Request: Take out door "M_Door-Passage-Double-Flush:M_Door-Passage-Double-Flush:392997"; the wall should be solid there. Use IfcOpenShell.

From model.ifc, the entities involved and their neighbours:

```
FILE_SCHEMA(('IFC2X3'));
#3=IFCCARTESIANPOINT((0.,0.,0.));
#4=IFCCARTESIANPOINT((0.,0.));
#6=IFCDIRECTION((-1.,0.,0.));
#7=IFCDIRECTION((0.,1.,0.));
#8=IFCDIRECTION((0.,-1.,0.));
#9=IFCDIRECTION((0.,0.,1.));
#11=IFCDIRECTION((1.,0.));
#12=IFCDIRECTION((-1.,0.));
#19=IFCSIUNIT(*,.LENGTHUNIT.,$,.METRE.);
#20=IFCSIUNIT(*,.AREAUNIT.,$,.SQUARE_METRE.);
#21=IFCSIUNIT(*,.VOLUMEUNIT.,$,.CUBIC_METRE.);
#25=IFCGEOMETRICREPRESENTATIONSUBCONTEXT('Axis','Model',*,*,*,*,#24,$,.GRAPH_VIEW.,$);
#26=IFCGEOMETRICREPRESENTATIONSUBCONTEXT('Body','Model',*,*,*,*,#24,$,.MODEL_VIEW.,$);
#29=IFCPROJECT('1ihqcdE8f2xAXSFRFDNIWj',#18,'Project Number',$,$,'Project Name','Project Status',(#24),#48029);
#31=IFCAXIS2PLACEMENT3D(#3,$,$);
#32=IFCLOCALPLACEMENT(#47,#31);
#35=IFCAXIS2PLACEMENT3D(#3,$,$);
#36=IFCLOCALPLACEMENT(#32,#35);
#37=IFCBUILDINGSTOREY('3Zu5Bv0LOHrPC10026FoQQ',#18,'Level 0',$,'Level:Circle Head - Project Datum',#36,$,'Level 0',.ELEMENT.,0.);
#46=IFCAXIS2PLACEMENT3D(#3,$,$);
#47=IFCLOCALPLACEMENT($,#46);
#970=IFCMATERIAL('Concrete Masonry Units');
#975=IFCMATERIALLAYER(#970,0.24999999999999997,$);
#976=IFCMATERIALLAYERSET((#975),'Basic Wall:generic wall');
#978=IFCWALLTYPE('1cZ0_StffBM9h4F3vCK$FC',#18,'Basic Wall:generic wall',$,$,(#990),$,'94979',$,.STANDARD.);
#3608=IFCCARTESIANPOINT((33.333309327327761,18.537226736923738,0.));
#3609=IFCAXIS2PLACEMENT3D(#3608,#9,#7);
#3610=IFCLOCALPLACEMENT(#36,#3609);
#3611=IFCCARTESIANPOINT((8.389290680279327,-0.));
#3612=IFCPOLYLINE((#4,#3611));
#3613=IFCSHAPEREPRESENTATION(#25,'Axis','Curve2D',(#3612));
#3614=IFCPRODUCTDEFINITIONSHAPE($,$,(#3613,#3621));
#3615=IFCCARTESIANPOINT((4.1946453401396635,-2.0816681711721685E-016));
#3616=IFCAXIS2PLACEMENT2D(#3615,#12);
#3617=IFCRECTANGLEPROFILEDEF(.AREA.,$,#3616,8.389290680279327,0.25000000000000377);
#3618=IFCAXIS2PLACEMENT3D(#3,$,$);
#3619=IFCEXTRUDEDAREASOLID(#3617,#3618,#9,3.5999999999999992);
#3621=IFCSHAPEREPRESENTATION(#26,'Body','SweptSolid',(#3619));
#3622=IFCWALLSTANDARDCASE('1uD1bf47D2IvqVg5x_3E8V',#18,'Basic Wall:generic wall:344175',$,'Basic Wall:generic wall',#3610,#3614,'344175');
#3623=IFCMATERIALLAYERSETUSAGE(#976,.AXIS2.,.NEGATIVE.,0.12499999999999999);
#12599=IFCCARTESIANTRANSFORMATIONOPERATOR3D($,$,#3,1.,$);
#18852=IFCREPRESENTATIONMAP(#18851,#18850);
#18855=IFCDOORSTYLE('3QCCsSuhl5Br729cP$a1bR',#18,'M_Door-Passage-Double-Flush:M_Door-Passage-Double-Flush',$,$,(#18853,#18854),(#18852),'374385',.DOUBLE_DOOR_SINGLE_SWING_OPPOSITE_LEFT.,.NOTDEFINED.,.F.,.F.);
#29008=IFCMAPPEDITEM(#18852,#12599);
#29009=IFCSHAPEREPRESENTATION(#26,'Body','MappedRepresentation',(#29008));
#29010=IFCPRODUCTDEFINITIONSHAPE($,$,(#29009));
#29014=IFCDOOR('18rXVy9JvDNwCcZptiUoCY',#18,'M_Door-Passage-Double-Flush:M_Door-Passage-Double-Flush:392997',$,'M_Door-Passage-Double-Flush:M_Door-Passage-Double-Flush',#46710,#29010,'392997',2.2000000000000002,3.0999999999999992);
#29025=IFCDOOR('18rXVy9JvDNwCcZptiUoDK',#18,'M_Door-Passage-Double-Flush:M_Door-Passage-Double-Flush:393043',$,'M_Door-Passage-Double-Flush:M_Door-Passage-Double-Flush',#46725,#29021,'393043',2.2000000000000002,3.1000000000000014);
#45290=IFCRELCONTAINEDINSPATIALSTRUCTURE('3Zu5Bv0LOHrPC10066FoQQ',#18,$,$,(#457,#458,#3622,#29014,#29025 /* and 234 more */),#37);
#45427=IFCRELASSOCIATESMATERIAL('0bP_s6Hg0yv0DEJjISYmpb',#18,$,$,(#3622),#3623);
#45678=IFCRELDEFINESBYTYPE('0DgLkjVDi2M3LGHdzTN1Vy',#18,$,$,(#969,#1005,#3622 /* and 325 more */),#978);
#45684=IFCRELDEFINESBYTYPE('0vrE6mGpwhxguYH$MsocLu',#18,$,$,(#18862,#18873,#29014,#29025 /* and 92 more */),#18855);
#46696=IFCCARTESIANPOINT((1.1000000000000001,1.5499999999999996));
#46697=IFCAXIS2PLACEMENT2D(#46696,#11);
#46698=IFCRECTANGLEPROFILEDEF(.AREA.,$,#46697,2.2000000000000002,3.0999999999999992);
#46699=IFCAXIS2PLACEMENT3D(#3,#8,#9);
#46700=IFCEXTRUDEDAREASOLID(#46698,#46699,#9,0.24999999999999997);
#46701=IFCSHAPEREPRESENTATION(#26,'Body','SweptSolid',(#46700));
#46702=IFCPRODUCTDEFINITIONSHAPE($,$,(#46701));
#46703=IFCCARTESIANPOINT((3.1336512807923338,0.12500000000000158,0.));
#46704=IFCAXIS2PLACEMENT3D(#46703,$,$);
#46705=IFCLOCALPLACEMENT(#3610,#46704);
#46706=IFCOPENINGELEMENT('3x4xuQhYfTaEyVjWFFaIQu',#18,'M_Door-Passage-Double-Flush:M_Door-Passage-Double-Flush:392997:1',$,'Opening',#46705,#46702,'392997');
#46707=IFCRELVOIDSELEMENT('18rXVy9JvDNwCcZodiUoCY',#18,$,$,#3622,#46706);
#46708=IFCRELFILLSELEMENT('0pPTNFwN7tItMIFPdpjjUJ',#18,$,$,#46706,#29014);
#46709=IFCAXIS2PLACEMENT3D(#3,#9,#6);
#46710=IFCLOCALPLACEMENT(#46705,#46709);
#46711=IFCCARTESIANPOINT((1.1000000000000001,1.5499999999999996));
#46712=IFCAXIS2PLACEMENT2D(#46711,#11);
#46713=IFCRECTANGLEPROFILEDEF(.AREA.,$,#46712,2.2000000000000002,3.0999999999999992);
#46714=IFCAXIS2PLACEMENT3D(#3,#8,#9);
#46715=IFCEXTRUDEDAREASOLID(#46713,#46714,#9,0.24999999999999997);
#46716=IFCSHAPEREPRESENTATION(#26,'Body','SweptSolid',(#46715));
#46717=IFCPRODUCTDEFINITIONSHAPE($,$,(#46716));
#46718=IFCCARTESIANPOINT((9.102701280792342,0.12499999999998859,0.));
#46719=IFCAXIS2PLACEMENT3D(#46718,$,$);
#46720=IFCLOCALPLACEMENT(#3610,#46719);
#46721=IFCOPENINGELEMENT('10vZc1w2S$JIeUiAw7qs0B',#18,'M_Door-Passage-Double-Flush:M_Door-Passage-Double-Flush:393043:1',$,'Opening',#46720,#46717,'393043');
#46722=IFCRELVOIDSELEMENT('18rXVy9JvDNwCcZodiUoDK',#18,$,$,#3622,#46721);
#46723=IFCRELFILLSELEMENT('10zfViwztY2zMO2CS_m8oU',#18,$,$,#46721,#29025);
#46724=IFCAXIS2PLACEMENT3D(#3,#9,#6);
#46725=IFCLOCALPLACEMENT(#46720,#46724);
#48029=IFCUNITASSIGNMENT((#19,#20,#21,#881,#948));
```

```python
import ifcopenshell
import ifcopenshell.api.feature
import ifcopenshell.api.root
import ifcopenshell.geom
import ifcopenshell.util.shape

model = ifcopenshell.open("model.ifc")
settings = ifcopenshell.geom.settings()


def volume(element):
    """Net volume in cubic metres, openings subtracted."""
    shape = ifcopenshell.geom.create_shape(settings, element)
    return ifcopenshell.util.shape.get_volume(shape.geometry)


door = model.by_guid("18rXVy9JvDNwCcZptiUoCY")
opening = door.FillsVoids[0].RelatingOpeningElement
wall = opening.VoidsElements[0].RelatingBuildingElement
before = volume(wall)

ifcopenshell.api.root.remove_product(model, product=door)
ifcopenshell.api.feature.remove_feature(model, feature=opening)

after = volume(wall)

print(f"wall volume {before:.3f} -> {after:.3f} m3")

model.write("model_rev.ifc")
```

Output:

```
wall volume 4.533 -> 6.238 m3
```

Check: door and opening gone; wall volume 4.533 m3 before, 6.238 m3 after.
